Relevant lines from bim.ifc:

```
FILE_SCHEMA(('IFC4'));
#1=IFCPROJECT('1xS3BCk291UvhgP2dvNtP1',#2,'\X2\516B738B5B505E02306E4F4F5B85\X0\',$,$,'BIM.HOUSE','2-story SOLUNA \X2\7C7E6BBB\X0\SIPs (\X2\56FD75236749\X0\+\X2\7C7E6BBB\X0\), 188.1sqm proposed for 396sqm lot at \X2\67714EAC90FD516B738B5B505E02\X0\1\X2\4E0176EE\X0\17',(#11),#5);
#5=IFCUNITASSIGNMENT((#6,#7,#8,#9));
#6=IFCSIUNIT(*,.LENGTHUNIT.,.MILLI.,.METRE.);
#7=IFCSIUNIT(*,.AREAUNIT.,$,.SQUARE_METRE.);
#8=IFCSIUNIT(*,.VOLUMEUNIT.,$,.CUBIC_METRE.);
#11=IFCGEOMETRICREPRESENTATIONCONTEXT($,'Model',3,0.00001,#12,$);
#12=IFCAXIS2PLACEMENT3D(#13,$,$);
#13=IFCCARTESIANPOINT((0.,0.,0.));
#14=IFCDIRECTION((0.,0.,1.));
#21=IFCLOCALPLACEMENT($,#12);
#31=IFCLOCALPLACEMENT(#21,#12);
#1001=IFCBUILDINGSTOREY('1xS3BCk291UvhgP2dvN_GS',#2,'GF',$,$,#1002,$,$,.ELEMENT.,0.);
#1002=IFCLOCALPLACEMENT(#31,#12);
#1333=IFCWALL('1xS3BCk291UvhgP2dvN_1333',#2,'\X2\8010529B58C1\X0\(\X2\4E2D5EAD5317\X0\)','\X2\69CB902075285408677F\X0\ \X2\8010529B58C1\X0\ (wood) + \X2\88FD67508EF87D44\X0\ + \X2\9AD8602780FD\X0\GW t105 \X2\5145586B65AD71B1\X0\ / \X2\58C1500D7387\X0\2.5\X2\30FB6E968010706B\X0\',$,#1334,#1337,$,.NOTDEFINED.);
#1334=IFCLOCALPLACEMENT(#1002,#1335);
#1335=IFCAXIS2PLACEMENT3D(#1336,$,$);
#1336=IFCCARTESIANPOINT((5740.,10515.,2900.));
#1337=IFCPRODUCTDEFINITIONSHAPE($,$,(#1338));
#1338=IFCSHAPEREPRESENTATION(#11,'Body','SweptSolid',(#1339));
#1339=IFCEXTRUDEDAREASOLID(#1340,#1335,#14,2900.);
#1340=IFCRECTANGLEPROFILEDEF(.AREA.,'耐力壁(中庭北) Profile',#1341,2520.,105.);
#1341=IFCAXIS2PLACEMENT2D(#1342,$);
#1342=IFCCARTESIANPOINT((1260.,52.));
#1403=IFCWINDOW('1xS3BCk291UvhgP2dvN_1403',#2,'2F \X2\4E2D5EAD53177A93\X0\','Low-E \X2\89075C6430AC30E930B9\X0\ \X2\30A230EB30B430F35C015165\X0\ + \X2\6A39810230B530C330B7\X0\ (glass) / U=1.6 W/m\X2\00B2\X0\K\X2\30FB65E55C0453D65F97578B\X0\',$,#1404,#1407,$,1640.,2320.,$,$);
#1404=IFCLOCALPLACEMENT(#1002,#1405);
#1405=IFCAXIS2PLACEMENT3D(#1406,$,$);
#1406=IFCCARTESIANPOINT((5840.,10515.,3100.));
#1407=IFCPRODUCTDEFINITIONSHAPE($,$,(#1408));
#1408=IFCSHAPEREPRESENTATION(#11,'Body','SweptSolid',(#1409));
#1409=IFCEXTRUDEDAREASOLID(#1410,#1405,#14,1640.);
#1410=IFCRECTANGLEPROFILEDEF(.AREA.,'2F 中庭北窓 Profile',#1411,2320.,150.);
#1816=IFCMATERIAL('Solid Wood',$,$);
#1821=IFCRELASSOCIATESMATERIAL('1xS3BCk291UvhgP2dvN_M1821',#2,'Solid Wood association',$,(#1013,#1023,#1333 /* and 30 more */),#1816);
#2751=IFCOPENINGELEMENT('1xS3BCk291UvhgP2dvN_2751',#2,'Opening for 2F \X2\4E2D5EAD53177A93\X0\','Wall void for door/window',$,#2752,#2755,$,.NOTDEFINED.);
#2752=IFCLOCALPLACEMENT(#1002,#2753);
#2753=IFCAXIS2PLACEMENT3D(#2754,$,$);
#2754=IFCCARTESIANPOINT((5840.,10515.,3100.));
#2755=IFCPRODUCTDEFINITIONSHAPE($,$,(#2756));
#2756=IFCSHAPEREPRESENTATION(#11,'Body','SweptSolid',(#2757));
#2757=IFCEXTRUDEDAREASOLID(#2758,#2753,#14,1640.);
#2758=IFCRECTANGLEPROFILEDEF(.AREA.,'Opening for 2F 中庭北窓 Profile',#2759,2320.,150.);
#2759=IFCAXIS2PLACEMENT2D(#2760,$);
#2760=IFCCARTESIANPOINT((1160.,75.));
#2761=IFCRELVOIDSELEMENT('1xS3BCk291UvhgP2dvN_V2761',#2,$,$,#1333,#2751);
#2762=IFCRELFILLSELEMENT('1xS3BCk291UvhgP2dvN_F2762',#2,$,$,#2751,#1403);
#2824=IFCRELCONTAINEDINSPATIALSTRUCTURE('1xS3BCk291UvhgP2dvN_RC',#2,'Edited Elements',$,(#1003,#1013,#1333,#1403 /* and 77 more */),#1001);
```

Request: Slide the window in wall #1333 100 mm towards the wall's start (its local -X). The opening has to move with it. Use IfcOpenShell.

```python
import ifcopenshell
import ifcopenshell.api.geometry
import ifcopenshell.util.placement

model = ifcopenshell.open("bim.ifc")

window = model.by_guid("1xS3BCk291UvhgP2dvN_1403")
opening = window.FillsVoids[0].RelatingOpeningElement
wall = opening.VoidsElements[0].RelatingBuildingElement

wall_matrix = ifcopenshell.util.placement.get_local_placement(wall.ObjectPlacement)
shift = wall_matrix[:3, 0] * -100.0
before = ifcopenshell.util.placement.get_local_placement(window.ObjectPlacement)[:3, 3].copy()

# The window is not placed relative to its opening, so move both.
for product in (opening, window):
    matrix = ifcopenshell.util.placement.get_local_placement(product.ObjectPlacement)
    matrix[:3, 3] += shift
    ifcopenshell.api.geometry.edit_object_placement(model, product=product, matrix=matrix, is_si=False)

after = ifcopenshell.util.placement.get_local_placement(window.ObjectPlacement)[:3, 3]
print("window moved by", (after - before).round(3) + 0.0)

model.write("bim-out.ifc")
```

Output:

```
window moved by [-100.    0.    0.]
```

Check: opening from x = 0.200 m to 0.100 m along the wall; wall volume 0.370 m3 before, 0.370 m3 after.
